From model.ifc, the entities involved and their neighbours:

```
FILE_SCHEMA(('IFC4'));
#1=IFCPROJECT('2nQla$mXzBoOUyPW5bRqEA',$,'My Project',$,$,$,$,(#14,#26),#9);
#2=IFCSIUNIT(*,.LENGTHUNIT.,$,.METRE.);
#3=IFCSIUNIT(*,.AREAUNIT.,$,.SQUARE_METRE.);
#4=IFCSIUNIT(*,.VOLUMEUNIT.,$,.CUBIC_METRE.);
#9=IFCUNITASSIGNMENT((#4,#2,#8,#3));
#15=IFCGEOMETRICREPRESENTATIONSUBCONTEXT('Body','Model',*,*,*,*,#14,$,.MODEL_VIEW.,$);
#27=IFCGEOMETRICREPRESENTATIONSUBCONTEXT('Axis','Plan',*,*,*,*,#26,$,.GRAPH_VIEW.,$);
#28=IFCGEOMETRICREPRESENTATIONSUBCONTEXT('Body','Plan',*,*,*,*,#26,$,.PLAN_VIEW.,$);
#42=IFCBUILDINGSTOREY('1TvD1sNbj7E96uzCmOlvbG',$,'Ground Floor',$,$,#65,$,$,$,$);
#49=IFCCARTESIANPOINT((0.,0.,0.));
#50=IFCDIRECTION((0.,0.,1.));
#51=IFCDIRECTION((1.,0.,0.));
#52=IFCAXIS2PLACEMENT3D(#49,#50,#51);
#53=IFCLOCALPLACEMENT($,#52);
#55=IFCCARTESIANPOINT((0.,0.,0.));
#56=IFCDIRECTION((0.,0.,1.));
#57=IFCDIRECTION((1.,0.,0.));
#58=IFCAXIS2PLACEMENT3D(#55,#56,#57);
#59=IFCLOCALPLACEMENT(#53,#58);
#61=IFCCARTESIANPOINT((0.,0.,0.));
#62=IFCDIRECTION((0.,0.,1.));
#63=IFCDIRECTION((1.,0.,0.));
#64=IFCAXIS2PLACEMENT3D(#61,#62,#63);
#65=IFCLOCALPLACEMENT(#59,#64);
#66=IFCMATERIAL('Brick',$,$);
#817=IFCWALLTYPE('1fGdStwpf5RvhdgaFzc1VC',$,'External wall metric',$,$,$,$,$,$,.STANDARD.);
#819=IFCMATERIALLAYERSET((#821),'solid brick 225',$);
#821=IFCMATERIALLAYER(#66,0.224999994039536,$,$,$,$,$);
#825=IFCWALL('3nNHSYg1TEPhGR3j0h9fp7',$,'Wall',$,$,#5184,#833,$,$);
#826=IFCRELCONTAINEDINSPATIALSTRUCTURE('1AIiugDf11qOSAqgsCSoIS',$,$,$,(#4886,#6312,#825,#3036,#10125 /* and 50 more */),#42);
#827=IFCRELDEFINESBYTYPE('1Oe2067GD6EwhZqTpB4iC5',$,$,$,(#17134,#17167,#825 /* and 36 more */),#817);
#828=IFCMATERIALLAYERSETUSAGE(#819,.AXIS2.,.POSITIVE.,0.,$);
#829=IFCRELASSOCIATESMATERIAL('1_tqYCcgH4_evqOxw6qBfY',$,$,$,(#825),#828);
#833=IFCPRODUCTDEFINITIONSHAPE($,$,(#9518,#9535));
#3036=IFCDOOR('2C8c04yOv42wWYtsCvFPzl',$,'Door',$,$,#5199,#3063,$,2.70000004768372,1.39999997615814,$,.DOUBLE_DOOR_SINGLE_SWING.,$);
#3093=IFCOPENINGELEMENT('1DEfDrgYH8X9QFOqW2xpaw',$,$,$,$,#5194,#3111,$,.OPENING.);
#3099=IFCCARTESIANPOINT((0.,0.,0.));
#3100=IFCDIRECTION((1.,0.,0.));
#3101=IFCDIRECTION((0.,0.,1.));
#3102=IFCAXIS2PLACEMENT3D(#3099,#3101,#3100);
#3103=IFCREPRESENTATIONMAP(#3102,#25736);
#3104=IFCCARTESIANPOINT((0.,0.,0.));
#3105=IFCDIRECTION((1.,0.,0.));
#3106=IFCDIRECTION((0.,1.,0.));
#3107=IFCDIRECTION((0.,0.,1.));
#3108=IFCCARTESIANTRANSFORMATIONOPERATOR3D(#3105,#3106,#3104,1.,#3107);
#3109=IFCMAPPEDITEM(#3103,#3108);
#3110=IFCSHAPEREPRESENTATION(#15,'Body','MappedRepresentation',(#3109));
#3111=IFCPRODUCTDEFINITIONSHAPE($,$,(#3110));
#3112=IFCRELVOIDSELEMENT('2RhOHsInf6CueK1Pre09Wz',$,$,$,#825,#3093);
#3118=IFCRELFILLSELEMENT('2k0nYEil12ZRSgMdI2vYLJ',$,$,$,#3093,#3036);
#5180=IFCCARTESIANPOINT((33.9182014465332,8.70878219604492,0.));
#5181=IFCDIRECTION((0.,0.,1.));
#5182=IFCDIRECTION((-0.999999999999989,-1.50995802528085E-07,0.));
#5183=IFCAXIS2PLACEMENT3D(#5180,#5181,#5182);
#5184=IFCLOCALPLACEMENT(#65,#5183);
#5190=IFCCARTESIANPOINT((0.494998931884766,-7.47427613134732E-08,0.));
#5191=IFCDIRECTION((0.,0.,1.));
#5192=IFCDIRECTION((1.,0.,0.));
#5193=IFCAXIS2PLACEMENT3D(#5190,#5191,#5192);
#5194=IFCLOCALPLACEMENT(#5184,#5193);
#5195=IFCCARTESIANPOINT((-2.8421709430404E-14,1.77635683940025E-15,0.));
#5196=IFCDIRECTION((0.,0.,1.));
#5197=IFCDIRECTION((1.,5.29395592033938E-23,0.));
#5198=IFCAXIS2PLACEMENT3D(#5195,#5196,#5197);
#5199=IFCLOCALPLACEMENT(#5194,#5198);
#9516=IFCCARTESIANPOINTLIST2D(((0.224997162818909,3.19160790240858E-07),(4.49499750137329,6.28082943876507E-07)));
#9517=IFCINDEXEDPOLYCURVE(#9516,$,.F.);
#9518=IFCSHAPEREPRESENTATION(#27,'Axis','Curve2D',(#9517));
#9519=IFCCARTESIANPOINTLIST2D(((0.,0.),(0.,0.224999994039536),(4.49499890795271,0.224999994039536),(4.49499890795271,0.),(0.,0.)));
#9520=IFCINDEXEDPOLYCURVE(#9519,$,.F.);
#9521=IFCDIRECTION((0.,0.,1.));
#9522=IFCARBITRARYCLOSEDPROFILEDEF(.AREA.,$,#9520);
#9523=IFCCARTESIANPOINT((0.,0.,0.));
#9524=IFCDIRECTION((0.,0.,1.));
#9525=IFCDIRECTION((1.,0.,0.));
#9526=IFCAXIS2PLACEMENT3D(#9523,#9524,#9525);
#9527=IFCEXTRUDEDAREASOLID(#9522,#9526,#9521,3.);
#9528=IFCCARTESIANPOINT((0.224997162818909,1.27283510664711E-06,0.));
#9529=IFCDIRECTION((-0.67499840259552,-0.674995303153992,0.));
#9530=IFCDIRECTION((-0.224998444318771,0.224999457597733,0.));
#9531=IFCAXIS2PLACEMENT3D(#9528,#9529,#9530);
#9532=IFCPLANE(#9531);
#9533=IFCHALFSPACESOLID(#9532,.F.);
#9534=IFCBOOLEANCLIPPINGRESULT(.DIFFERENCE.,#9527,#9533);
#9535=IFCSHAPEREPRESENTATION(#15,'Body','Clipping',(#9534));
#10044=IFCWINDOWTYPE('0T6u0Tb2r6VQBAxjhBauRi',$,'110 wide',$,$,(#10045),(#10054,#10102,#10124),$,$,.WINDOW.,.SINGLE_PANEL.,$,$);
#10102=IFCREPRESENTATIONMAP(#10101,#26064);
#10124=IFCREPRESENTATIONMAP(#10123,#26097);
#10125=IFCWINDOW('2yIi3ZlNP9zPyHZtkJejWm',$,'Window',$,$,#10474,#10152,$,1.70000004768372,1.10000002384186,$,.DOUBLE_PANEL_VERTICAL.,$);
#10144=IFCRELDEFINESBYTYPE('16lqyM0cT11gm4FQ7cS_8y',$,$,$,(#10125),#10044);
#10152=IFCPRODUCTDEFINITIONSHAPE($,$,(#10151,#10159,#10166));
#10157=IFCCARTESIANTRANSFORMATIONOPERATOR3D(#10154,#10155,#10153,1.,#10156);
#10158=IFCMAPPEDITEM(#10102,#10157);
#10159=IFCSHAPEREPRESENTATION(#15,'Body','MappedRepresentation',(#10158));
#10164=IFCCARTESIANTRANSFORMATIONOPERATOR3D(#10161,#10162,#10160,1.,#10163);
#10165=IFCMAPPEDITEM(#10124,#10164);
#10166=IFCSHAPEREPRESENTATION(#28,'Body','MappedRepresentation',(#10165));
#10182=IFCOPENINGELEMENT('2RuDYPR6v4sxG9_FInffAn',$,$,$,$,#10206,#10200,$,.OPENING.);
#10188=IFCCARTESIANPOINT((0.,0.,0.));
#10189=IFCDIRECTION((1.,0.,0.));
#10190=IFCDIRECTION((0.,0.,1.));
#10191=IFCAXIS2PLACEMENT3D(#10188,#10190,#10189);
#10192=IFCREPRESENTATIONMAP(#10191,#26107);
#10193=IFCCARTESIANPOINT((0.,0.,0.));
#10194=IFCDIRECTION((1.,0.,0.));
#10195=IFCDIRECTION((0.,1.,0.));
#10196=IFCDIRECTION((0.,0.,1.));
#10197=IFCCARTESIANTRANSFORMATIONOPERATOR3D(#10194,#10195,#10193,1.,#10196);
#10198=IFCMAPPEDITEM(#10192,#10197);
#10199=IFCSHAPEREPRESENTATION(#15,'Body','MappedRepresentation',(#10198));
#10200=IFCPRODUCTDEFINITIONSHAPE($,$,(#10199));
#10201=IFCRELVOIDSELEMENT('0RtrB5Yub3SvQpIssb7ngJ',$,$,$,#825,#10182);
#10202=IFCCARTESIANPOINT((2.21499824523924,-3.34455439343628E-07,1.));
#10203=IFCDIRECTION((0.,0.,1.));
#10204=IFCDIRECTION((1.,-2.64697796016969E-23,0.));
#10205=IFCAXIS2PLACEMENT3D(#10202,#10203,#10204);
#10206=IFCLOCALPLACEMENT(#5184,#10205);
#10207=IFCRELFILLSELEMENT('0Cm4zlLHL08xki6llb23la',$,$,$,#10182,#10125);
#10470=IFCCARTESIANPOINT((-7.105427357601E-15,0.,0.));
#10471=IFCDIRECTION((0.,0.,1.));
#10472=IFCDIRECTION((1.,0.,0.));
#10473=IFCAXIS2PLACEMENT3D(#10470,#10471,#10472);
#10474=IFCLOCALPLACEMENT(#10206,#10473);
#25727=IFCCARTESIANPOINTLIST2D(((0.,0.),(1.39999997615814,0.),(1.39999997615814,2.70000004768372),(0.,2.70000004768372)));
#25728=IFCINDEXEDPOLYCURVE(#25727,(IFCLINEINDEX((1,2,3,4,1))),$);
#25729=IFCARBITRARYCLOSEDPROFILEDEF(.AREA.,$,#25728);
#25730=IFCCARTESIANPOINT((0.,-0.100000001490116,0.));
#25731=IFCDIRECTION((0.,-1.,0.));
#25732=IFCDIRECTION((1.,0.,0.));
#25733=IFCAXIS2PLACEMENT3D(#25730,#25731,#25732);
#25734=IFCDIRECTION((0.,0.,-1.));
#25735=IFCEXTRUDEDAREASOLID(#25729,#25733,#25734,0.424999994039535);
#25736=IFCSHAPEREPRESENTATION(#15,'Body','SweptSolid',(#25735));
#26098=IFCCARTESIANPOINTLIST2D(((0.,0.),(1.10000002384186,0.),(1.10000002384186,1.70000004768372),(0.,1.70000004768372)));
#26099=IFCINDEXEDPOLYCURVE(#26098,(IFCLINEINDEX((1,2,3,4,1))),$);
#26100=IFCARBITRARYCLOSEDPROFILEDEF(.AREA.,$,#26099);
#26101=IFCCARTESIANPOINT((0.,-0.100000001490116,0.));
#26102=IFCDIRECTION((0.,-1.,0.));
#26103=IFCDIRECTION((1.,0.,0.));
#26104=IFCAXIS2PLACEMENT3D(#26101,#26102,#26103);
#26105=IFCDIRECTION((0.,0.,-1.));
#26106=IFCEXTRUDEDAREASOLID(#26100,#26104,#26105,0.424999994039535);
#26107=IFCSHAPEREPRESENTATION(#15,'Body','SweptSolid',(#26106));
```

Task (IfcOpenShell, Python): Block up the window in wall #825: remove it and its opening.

```python
import ifcopenshell
import ifcopenshell.api.feature
import ifcopenshell.api.root
import ifcopenshell.geom
import ifcopenshell.util.shape

model = ifcopenshell.open("model.ifc")
settings = ifcopenshell.geom.settings()


def volume(element):
    """Net volume in cubic metres, openings subtracted."""
    shape = ifcopenshell.geom.create_shape(settings, element)
    return ifcopenshell.util.shape.get_volume(shape.geometry)


window = model.by_guid("2yIi3ZlNP9zPyHZtkJejWm")
opening = window.FillsVoids[0].RelatingOpeningElement
wall = opening.VoidsElements[0].RelatingBuildingElement
before = volume(wall)

ifcopenshell.api.root.remove_product(model, product=window)
ifcopenshell.api.feature.remove_feature(model, feature=opening)

after = volume(wall)

print(f"wall volume {before:.3f} -> {after:.3f} m3")

model.write("model-out.ifc")
```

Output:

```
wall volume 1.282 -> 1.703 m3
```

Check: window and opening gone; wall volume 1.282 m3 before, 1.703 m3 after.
